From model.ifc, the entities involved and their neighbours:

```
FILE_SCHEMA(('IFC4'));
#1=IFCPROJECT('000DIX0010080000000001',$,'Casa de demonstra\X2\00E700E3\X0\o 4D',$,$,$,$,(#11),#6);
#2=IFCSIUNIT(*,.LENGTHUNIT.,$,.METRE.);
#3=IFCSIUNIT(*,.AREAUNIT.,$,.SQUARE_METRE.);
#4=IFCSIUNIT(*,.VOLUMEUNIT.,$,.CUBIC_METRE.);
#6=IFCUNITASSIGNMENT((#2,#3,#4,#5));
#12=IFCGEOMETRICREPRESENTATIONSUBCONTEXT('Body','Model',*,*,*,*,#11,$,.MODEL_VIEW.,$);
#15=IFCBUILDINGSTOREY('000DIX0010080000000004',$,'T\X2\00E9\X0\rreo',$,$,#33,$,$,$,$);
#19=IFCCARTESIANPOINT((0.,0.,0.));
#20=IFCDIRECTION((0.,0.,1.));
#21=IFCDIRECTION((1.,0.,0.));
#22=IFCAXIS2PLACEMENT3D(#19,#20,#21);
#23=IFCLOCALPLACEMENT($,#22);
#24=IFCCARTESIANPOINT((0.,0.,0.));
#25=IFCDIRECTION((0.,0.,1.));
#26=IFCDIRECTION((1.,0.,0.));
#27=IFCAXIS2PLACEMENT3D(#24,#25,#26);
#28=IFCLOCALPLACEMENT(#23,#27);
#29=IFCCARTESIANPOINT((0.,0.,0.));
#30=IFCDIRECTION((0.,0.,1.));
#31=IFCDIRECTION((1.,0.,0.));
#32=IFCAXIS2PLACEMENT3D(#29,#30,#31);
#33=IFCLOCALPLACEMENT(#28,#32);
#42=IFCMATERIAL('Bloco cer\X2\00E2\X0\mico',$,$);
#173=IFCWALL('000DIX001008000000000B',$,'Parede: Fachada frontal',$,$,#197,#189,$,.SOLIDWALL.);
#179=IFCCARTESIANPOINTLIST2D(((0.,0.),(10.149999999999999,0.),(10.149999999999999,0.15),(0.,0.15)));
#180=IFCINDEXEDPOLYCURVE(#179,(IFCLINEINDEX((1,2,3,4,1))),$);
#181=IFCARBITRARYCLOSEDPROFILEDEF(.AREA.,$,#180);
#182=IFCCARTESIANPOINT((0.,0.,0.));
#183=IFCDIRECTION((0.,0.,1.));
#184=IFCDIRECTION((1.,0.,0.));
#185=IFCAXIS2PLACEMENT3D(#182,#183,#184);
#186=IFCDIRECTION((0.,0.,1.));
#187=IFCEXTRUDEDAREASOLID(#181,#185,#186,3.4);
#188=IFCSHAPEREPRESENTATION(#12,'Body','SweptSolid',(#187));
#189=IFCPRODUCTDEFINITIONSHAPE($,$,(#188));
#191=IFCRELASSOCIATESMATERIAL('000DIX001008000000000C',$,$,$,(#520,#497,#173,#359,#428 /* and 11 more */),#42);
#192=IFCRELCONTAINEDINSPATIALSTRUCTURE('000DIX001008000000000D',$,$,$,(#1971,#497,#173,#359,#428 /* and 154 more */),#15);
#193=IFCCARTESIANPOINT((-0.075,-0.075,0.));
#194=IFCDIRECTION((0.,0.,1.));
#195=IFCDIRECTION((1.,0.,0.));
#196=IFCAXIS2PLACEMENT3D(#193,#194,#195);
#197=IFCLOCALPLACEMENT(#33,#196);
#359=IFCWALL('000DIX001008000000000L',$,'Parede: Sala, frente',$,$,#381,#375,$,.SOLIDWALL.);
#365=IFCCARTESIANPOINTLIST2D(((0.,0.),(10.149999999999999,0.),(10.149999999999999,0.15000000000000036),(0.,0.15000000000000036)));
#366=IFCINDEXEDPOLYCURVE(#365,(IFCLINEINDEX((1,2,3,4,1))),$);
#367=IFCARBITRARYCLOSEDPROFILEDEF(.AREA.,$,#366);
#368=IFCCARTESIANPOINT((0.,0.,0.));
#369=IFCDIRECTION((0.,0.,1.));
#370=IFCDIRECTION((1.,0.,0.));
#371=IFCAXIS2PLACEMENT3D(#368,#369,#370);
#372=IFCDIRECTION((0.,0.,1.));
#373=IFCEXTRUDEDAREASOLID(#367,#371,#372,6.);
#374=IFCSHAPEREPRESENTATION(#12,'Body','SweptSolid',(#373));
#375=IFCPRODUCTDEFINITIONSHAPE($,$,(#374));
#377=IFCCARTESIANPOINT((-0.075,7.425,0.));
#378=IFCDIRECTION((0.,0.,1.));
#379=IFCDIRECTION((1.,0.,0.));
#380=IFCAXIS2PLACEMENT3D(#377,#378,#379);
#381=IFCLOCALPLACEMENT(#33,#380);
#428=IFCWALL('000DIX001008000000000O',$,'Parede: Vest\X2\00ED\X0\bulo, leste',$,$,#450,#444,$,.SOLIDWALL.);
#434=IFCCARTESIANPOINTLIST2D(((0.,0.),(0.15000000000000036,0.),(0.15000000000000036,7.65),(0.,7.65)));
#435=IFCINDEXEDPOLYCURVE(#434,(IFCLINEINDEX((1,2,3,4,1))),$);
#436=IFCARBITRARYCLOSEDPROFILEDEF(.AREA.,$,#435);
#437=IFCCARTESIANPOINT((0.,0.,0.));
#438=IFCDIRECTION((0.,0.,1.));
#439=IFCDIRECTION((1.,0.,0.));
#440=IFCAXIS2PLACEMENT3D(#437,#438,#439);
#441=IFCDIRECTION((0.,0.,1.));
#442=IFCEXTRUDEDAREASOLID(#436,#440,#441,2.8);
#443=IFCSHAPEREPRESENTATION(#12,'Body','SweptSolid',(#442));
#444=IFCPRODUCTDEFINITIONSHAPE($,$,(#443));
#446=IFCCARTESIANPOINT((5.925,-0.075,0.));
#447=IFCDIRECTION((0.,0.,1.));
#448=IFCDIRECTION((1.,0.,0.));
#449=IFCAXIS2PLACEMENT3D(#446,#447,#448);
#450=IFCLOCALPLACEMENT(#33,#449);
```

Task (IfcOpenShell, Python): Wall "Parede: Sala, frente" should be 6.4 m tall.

```python
import ifcopenshell
import ifcopenshell.geom
import ifcopenshell.util.representation
import ifcopenshell.util.shape

model = ifcopenshell.open("model.ifc")
settings = ifcopenshell.geom.settings()


def volume(element):
    """Net volume in cubic metres, openings subtracted."""
    shape = ifcopenshell.geom.create_shape(settings, element)
    return ifcopenshell.util.shape.get_volume(shape.geometry)


wall = model.by_guid("000DIX001008000000000L")
before = volume(wall)

body = ifcopenshell.util.representation.get_representation(wall, "Model", "Body")
solid = body.Items[0]
old_height = solid.Depth
solid.Depth = 6.4
after = volume(wall)

print(f"height {old_height:g} -> {solid.Depth:g}, volume {before:.3f} -> {after:.3f} m3")

model.write("model_rev.ifc")
```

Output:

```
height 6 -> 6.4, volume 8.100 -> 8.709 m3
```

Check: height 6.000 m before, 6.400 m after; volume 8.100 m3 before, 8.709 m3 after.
